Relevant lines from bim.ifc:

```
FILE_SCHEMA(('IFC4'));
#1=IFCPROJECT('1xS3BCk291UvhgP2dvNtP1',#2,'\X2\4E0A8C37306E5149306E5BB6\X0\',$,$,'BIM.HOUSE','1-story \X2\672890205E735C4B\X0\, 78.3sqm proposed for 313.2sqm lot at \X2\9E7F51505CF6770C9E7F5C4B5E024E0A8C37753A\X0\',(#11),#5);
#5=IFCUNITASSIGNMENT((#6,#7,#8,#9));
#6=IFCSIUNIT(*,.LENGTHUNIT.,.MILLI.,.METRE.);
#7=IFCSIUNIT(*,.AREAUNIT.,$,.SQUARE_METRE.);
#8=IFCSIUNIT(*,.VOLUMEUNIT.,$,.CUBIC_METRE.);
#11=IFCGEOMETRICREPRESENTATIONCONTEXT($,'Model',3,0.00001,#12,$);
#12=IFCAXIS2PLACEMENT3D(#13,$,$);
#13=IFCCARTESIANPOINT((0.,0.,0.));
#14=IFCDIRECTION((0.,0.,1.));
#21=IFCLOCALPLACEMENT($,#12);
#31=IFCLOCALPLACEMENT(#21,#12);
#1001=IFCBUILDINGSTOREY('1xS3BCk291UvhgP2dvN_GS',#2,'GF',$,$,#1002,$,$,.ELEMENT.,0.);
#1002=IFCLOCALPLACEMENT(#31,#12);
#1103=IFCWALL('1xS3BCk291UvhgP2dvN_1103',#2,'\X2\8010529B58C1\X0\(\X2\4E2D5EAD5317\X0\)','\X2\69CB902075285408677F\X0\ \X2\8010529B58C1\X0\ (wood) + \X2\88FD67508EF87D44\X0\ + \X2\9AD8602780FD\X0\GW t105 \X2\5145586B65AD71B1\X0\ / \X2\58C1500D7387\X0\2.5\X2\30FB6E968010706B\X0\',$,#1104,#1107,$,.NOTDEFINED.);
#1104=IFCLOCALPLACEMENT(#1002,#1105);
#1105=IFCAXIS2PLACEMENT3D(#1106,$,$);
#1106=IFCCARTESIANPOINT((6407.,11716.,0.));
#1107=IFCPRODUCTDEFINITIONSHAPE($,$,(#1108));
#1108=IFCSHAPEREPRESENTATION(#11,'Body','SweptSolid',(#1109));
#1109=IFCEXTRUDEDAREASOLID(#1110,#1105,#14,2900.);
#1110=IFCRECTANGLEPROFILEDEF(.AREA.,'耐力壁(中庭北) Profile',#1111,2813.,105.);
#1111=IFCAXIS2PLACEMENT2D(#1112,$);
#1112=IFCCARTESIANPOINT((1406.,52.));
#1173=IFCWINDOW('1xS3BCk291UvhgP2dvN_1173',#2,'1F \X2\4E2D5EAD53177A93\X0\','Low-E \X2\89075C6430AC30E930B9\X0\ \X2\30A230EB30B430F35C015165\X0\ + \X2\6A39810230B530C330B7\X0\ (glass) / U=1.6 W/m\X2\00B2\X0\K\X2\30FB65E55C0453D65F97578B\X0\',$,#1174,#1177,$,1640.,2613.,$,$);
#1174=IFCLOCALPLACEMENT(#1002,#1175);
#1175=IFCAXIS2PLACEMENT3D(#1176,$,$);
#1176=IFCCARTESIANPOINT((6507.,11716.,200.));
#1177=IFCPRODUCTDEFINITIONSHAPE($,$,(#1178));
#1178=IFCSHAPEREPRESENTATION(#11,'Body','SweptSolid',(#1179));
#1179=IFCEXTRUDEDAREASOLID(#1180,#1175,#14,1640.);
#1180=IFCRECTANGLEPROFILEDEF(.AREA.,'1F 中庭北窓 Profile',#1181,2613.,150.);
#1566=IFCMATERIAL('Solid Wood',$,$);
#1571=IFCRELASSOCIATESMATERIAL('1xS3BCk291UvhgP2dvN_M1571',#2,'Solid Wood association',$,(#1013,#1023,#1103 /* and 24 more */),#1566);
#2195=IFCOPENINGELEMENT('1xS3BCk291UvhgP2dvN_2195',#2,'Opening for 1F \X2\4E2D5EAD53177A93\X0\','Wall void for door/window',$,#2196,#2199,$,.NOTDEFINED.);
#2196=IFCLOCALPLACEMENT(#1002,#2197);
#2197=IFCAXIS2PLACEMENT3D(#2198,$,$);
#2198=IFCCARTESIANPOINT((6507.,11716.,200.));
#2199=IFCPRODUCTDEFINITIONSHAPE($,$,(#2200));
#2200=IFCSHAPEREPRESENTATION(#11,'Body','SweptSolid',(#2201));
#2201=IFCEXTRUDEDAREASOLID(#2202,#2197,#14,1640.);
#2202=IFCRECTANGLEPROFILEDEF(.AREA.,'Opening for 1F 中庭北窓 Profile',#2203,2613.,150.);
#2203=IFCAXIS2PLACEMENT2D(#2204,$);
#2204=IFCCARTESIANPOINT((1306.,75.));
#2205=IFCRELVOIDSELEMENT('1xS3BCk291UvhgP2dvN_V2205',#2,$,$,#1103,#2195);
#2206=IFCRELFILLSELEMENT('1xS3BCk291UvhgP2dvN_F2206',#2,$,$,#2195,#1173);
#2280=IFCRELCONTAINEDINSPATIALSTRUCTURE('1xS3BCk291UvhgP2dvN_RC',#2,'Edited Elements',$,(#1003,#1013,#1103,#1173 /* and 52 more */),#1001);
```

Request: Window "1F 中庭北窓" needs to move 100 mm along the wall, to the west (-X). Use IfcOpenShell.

```python
import ifcopenshell
import ifcopenshell.api.geometry
import ifcopenshell.util.placement
import ifcopenshell.util.unit

model = ifcopenshell.open("bim.ifc")
unit_scale = ifcopenshell.util.unit.calculate_unit_scale(model)

window = model.by_guid("1xS3BCk291UvhgP2dvN_1173")
opening = window.FillsVoids[0].RelatingOpeningElement
wall = opening.VoidsElements[0].RelatingBuildingElement

wall_matrix = ifcopenshell.util.placement.get_local_placement(wall.ObjectPlacement)
shift = wall_matrix[:3, 0] * -0.1 / unit_scale
before = ifcopenshell.util.placement.get_local_placement(window.ObjectPlacement)[:3, 3].copy()

# The window is not placed relative to its opening, so move both.
for product in (opening, window):
    matrix = ifcopenshell.util.placement.get_local_placement(product.ObjectPlacement)
    matrix[:3, 3] += shift
    ifcopenshell.api.geometry.edit_object_placement(model, product=product, matrix=matrix, is_si=False)

after = ifcopenshell.util.placement.get_local_placement(window.ObjectPlacement)[:3, 3]
print("window moved by", (after - before).round(3) + 0.0)

model.write("bim-out.ifc")
```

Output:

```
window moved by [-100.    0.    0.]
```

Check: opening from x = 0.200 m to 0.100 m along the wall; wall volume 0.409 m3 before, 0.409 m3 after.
